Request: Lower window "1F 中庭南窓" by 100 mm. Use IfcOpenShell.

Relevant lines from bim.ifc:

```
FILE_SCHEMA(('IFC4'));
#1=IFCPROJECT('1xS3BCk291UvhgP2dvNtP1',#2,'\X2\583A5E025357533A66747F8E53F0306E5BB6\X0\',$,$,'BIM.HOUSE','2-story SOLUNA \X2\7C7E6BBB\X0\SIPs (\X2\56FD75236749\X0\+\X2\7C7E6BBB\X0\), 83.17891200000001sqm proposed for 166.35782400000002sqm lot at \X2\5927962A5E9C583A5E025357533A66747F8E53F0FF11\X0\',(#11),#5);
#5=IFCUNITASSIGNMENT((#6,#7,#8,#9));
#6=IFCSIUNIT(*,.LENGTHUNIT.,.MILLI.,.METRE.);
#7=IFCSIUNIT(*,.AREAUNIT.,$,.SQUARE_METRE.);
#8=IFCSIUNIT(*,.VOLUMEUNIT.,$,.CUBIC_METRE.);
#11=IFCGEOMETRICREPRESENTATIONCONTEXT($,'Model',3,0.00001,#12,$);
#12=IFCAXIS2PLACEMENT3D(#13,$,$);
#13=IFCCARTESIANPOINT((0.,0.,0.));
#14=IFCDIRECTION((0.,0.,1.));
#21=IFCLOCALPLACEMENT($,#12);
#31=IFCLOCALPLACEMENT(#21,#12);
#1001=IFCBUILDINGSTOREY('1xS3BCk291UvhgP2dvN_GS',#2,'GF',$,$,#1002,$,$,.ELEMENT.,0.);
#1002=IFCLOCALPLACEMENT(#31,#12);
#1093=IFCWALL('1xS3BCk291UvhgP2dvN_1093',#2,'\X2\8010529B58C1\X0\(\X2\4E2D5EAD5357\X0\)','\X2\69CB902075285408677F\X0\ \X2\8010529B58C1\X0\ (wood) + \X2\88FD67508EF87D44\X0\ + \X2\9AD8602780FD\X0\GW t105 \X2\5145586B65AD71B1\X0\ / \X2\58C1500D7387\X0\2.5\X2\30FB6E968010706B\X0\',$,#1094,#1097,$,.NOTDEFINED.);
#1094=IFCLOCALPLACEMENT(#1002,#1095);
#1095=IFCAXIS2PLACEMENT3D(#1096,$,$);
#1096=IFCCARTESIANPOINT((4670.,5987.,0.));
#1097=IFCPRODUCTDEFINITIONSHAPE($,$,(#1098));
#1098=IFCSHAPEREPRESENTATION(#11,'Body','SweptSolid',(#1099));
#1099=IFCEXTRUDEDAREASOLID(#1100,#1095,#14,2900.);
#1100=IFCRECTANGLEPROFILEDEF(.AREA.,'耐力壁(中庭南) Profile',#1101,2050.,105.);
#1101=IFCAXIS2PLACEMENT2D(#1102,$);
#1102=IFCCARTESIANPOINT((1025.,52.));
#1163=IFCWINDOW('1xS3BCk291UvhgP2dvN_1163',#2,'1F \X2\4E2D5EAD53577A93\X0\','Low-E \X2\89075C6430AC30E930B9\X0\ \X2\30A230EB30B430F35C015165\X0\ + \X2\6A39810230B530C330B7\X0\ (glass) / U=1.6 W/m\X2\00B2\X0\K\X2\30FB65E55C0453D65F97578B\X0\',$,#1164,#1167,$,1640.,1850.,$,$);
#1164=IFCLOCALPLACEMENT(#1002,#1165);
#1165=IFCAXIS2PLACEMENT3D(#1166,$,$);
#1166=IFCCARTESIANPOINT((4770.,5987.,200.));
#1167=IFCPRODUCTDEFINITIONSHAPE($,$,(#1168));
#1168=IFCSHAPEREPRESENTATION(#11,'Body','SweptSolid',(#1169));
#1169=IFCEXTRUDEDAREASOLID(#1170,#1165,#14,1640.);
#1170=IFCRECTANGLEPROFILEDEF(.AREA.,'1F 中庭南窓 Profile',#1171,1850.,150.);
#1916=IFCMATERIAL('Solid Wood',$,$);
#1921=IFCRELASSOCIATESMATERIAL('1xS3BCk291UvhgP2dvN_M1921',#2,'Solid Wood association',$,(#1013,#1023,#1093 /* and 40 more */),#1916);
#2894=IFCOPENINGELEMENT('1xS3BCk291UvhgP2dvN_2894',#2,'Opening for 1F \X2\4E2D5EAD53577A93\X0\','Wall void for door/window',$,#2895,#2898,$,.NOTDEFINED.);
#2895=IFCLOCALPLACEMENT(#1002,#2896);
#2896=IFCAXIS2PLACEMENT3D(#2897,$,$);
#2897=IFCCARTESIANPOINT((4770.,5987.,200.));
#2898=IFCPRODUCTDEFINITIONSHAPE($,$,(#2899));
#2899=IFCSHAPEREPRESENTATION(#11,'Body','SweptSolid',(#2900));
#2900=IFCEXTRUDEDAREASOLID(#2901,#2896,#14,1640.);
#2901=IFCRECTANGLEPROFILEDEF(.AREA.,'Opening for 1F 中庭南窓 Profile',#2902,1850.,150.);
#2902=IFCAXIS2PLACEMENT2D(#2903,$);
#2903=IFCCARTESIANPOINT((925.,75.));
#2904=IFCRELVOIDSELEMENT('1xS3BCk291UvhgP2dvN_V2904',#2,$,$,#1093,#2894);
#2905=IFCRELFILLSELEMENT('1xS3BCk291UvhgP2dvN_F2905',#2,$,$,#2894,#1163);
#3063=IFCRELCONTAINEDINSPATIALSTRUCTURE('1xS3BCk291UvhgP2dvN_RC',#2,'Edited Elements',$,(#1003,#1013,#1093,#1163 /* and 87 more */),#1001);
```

```python
import numpy as np
import ifcopenshell
import ifcopenshell.api.geometry
import ifcopenshell.util.placement
import ifcopenshell.util.unit

model = ifcopenshell.open("bim.ifc")
unit_scale = ifcopenshell.util.unit.calculate_unit_scale(model)

window = model.by_guid("1xS3BCk291UvhgP2dvN_1163")
opening = window.FillsVoids[0].RelatingOpeningElement
dz = -100.0

shift = np.array([0.0, 0.0, dz])
# The window is not placed relative to its opening, so move both.
for product in (opening, window):
    matrix = ifcopenshell.util.placement.get_local_placement(product.ObjectPlacement)
    matrix[:3, 3] += shift
    ifcopenshell.api.geometry.edit_object_placement(model, product=product, matrix=matrix, is_si=False)

print(f"moved by {dz * unit_scale:+.3f} m")

model.write("bim_v2.ifc")
```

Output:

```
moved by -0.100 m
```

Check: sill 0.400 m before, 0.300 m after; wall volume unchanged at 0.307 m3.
